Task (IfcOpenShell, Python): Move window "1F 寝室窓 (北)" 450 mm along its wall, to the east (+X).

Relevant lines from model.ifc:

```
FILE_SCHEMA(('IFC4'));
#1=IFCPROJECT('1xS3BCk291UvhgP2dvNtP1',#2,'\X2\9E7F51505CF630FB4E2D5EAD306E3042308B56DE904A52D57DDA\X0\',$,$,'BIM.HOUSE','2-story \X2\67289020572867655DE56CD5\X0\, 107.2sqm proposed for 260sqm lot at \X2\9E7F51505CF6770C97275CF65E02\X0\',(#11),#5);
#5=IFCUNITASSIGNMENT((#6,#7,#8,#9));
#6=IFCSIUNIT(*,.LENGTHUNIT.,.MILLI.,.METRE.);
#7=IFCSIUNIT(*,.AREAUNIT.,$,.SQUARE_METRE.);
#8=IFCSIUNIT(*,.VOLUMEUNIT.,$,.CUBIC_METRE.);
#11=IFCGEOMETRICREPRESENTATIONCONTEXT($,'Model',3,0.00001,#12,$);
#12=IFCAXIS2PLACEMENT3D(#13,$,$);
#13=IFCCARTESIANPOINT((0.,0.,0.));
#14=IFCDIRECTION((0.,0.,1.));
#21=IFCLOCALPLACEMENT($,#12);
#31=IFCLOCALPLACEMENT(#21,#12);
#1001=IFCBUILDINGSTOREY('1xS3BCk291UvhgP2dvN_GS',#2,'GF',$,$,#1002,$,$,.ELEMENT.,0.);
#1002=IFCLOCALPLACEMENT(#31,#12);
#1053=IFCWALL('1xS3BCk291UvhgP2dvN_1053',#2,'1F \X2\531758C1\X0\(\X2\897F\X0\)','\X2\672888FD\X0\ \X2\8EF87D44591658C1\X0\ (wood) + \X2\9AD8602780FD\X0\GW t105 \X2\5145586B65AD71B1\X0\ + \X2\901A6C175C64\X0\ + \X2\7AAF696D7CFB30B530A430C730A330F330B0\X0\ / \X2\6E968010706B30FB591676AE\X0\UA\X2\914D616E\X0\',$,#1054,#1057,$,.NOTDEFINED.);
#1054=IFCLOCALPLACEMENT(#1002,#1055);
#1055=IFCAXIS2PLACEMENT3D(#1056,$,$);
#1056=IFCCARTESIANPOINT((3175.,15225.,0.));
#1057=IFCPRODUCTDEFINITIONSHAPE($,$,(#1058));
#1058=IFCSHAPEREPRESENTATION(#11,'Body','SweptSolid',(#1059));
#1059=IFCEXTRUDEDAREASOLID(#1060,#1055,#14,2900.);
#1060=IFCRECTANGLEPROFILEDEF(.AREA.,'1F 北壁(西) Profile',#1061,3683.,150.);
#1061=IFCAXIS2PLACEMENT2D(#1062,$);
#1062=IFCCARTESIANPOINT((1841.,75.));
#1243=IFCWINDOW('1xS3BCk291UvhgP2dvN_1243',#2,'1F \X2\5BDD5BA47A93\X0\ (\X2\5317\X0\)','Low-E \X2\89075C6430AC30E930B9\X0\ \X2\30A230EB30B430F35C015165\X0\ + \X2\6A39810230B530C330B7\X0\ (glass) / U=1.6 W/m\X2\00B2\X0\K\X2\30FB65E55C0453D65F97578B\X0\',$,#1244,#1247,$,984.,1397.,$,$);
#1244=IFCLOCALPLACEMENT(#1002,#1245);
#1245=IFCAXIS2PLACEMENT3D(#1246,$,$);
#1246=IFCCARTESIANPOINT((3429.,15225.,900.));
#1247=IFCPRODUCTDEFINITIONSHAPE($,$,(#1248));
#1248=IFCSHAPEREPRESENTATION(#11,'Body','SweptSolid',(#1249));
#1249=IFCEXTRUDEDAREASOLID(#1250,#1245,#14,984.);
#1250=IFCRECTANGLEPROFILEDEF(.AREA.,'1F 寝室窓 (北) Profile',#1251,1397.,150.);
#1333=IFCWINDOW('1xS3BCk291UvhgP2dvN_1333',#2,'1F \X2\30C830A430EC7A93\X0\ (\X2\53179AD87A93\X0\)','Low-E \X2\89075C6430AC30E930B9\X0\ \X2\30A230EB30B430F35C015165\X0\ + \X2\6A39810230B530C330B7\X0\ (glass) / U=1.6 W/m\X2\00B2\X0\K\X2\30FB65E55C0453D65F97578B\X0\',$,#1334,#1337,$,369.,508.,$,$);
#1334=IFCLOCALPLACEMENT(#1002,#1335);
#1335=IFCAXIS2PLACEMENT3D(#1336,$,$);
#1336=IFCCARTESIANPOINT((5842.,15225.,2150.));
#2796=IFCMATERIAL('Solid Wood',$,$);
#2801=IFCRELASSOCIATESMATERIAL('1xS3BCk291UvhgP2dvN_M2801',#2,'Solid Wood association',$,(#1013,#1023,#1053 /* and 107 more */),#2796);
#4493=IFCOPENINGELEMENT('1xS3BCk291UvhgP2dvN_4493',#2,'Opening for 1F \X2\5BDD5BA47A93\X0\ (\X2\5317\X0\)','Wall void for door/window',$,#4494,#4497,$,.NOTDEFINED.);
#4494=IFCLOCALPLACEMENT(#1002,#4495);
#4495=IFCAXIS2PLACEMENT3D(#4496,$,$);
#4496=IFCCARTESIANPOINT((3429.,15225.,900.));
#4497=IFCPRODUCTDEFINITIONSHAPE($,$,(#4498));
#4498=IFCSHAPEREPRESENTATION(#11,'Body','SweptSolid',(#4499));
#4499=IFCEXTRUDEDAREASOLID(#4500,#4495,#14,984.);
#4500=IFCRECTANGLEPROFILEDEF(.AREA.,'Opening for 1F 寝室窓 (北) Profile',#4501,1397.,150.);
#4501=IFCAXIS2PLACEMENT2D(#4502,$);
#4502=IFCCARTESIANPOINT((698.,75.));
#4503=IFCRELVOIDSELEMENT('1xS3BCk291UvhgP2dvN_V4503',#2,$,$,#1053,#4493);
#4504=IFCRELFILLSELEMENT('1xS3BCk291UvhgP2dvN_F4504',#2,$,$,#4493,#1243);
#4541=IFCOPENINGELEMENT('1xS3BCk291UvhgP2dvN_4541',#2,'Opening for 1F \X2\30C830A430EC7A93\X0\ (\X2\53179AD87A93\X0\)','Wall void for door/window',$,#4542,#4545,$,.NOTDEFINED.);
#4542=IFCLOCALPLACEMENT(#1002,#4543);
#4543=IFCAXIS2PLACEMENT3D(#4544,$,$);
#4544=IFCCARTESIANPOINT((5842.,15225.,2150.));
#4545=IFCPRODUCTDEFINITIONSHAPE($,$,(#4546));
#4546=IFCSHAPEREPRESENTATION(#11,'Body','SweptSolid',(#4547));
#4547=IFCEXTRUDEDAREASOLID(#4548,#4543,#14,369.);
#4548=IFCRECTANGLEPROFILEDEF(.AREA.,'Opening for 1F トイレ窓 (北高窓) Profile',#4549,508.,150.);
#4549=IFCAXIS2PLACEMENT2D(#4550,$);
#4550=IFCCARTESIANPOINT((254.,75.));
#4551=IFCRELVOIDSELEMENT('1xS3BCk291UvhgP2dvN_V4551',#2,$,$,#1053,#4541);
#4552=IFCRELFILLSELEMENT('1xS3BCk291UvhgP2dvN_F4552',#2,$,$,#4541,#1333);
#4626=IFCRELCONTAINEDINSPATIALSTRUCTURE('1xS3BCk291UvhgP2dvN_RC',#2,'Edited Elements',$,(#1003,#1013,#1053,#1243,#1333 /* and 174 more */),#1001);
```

```python
import ifcopenshell
import ifcopenshell.api.geometry
import ifcopenshell.util.placement
import ifcopenshell.util.unit

model = ifcopenshell.open("model.ifc")
unit_scale = ifcopenshell.util.unit.calculate_unit_scale(model)

window = model.by_id(1243)
opening = window.FillsVoids[0].RelatingOpeningElement
wall = opening.VoidsElements[0].RelatingBuildingElement

wall_matrix = ifcopenshell.util.placement.get_local_placement(wall.ObjectPlacement)
shift = wall_matrix[:3, 0] * 0.45 / unit_scale
before = ifcopenshell.util.placement.get_local_placement(window.ObjectPlacement)[:3, 3].copy()

# The window is not placed relative to its opening, so move both.
for product in (opening, window):
    matrix = ifcopenshell.util.placement.get_local_placement(product.ObjectPlacement)
    matrix[:3, 3] += shift
    ifcopenshell.api.geometry.edit_object_placement(model, product=product, matrix=matrix, is_si=False)

after = ifcopenshell.util.placement.get_local_placement(window.ObjectPlacement)[:3, 3]
print("window moved by", (after - before).round(3) + 0.0)

model.write("model_v2.ifc")
```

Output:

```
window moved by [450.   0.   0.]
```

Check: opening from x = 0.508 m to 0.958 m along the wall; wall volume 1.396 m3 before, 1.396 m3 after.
